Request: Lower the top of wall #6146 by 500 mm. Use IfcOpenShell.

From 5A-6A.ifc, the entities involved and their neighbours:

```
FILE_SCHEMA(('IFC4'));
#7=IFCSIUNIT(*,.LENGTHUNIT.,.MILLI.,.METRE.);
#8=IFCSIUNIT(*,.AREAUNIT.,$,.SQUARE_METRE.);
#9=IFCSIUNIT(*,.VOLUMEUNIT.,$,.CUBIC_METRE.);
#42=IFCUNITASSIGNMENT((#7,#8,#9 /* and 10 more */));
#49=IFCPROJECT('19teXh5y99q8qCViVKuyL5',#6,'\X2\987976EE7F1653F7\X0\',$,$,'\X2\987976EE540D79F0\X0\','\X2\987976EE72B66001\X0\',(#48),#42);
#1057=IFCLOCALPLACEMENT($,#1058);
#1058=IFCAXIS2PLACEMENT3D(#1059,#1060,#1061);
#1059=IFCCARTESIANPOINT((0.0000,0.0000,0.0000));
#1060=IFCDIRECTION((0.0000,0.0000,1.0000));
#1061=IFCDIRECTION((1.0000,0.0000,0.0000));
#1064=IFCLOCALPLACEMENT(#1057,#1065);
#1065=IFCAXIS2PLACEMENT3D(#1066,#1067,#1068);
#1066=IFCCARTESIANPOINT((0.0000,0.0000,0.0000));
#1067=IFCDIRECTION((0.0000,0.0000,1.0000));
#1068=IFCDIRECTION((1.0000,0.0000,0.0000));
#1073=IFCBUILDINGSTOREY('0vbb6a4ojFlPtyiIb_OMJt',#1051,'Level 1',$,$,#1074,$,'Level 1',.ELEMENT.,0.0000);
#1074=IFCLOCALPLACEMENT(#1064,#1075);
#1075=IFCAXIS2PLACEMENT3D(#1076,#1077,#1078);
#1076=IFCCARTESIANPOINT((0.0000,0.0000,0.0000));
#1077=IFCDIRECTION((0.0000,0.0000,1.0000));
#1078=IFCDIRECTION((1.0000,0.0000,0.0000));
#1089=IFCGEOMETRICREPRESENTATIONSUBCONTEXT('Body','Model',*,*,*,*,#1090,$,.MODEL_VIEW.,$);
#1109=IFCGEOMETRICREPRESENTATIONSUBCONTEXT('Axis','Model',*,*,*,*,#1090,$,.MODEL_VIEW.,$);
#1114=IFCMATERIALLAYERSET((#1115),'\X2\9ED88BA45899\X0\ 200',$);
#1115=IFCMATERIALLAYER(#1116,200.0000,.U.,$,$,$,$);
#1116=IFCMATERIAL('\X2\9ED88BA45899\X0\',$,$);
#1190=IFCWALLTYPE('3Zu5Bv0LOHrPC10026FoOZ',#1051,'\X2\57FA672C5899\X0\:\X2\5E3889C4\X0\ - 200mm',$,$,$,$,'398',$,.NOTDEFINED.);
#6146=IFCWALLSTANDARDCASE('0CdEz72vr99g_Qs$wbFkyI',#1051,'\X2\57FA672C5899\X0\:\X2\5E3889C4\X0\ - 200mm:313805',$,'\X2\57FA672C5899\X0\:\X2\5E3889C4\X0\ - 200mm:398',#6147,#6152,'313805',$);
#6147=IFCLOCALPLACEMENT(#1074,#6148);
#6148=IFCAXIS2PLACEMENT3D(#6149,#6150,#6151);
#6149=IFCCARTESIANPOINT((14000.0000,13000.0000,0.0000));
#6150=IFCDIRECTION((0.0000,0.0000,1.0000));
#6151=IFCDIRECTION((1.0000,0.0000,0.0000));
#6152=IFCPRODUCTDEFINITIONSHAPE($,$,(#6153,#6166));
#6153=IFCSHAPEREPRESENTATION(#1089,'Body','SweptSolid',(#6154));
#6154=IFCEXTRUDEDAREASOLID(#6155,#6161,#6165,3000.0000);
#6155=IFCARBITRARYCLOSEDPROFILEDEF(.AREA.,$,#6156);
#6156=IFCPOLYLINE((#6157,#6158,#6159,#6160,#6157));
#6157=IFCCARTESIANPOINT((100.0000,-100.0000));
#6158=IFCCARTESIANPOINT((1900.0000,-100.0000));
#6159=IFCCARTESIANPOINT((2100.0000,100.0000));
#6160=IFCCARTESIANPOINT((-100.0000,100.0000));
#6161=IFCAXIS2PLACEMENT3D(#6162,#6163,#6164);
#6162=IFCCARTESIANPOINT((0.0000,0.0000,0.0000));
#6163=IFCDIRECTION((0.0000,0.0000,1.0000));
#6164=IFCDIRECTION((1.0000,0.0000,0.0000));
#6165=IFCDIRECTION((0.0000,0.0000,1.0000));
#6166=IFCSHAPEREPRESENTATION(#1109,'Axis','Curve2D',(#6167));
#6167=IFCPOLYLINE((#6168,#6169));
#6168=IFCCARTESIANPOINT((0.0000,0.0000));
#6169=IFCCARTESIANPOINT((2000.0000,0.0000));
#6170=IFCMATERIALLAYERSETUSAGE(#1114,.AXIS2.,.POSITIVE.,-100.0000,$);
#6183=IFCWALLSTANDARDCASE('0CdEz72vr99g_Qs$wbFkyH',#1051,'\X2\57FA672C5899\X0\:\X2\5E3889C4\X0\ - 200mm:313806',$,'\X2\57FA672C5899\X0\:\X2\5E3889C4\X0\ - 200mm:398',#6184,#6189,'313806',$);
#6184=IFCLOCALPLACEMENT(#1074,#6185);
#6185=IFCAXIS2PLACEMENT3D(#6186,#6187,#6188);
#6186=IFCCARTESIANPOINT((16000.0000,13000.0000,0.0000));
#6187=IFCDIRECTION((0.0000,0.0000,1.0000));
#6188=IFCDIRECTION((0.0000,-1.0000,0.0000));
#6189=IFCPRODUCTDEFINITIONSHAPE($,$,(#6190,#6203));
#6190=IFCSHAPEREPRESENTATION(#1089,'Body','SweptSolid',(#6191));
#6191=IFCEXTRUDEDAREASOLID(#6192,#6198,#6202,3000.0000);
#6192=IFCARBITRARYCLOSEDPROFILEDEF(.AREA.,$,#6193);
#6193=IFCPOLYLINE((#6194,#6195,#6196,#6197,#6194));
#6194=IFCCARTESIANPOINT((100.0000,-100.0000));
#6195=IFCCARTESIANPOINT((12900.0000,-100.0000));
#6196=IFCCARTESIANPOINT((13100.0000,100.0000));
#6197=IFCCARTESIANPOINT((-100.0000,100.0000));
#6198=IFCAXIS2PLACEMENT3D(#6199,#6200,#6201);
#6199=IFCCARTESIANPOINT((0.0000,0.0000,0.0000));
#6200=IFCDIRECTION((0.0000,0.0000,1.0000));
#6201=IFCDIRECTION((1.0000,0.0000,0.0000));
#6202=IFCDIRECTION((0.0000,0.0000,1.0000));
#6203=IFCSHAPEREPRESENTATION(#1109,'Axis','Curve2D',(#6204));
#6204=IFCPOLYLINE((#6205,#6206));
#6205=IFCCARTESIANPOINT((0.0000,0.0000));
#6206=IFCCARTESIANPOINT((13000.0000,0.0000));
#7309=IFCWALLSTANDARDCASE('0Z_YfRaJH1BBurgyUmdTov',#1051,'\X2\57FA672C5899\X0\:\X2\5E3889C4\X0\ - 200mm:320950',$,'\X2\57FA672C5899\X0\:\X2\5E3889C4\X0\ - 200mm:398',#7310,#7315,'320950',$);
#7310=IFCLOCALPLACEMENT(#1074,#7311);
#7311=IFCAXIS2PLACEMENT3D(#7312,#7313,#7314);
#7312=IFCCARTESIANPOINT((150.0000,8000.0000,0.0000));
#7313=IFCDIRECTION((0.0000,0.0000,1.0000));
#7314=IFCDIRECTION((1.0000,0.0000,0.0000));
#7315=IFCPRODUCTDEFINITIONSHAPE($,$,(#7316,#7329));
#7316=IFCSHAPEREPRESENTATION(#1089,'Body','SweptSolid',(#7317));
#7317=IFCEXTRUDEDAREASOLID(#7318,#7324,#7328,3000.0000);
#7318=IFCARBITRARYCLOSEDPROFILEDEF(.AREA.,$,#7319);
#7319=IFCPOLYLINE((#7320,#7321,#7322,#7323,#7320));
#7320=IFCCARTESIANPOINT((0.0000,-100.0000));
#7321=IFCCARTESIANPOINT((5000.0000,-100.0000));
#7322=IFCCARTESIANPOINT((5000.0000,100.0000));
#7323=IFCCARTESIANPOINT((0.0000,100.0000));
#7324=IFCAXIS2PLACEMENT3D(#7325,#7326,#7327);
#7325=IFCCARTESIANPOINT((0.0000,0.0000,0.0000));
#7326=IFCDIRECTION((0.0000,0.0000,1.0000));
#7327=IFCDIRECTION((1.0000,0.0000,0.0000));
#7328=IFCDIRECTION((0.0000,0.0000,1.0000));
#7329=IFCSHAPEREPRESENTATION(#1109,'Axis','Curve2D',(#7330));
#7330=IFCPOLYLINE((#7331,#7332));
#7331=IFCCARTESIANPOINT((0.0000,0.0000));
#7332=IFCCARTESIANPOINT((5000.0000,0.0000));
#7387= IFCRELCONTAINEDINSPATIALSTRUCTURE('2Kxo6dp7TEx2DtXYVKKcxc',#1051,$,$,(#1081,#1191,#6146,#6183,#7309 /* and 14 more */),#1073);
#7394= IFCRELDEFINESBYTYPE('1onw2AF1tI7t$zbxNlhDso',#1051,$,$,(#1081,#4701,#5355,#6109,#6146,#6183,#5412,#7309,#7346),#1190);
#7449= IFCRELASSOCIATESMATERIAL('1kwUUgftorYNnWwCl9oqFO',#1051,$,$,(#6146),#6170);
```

```python
import ifcopenshell
import ifcopenshell.geom
import ifcopenshell.util.representation
import ifcopenshell.util.shape
import ifcopenshell.util.unit

model = ifcopenshell.open("5A-6A.ifc")
unit_scale = ifcopenshell.util.unit.calculate_unit_scale(model)
settings = ifcopenshell.geom.settings()


def volume(element):
    """Net volume in cubic metres, openings subtracted."""
    shape = ifcopenshell.geom.create_shape(settings, element)
    return ifcopenshell.util.shape.get_volume(shape.geometry)


wall = model.by_guid("0CdEz72vr99g_Qs$wbFkyI")
before = volume(wall)

body = ifcopenshell.util.representation.get_representation(wall, "Model", "Body")
solid = body.Items[0]
old_height = solid.Depth
solid.Depth -= 0.5 / unit_scale
after = volume(wall)

print(f"height {old_height:g} -> {solid.Depth:g}, volume {before:.3f} -> {after:.3f} m3")

model.write("5A-6A_v2.ifc")
```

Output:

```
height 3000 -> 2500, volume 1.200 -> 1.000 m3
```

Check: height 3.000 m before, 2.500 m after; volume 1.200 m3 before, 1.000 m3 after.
